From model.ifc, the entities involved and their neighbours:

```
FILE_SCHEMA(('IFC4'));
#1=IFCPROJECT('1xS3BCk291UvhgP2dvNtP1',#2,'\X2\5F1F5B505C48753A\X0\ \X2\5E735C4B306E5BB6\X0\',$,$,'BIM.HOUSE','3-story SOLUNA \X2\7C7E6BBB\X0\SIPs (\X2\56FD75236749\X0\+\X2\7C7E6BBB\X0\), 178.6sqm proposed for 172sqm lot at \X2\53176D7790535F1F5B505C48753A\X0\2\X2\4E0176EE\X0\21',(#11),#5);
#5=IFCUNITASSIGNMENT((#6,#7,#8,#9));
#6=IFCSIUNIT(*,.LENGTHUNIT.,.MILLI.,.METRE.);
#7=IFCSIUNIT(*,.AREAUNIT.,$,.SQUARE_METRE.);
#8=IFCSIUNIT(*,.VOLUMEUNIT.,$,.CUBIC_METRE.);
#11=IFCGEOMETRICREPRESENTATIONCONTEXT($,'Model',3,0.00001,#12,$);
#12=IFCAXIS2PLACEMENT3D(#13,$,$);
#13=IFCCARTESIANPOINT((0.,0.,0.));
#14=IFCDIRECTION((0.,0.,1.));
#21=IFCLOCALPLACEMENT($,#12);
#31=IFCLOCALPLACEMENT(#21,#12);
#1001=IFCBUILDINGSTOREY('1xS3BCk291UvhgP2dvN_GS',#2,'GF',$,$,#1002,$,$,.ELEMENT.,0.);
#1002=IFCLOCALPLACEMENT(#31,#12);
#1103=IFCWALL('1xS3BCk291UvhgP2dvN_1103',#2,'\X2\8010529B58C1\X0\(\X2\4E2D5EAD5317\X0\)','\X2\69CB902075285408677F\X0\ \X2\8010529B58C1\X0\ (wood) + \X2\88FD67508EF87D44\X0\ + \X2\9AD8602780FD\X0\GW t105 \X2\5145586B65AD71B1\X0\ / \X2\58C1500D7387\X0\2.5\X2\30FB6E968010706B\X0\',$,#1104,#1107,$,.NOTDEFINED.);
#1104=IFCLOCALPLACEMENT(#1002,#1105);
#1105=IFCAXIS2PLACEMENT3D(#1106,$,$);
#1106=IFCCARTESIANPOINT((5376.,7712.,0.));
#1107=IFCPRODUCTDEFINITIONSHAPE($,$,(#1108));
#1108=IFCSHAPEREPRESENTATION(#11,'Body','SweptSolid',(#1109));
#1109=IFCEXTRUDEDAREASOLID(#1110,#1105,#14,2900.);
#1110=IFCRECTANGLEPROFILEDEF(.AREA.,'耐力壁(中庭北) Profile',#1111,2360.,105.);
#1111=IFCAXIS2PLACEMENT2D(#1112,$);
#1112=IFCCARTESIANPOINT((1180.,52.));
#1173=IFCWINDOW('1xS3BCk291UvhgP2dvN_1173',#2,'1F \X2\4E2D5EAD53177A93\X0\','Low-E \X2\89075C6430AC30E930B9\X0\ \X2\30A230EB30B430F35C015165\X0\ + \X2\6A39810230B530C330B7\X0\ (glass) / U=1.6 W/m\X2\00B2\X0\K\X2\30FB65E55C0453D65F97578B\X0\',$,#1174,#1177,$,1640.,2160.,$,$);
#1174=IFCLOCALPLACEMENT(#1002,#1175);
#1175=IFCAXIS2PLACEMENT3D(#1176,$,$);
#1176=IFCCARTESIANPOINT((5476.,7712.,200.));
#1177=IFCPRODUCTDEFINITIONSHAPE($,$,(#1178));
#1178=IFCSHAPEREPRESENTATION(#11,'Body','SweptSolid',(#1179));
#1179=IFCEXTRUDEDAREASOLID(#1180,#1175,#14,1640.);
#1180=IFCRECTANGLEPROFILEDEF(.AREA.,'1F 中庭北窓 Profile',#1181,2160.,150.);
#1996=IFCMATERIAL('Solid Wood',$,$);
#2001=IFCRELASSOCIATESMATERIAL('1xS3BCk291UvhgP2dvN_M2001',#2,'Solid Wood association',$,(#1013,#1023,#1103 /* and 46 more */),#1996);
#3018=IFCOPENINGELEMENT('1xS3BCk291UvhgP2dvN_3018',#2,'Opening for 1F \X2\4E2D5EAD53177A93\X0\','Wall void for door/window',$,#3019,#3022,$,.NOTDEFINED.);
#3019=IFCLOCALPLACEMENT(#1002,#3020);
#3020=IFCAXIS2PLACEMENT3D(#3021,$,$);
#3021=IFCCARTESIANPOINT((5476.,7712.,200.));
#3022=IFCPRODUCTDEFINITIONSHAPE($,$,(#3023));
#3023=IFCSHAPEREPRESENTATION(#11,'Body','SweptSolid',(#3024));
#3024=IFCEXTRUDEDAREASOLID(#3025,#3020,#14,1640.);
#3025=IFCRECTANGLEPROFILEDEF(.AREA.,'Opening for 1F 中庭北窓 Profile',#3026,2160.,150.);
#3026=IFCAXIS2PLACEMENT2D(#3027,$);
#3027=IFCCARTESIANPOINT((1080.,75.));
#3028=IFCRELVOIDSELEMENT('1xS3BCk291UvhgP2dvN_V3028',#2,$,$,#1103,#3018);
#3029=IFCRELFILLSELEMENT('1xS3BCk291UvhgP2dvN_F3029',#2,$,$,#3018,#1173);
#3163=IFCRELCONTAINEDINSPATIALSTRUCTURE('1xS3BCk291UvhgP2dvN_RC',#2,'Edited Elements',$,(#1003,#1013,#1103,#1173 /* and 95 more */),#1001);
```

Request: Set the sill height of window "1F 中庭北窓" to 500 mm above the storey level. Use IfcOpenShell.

```python
import numpy as np
import ifcopenshell
import ifcopenshell.api.geometry
import ifcopenshell.geom
import ifcopenshell.util.element
import ifcopenshell.util.placement
import ifcopenshell.util.shape
import ifcopenshell.util.unit

model = ifcopenshell.open("model.ifc")
unit_scale = ifcopenshell.util.unit.calculate_unit_scale(model)

window = model.by_guid("1xS3BCk291UvhgP2dvN_1173")
opening = window.FillsVoids[0].RelatingOpeningElement
storey = ifcopenshell.util.element.get_container(window, ifc_class="IfcBuildingStorey")
level = ifcopenshell.util.placement.get_local_placement(storey.ObjectPlacement)[2, 3]

# The opening's origin need not be at the sill, so measure its lowest point.
shape = ifcopenshell.geom.create_shape(ifcopenshell.geom.settings(), opening)
bottom = ifcopenshell.util.shape.get_shape_bottom_elevation(shape, shape.geometry) / unit_scale
dz = level + 0.5 / unit_scale - bottom

shift = np.array([0.0, 0.0, dz])
# The window is not placed relative to its opening, so move both.
for product in (opening, window):
    matrix = ifcopenshell.util.placement.get_local_placement(product.ObjectPlacement)
    matrix[:3, 3] += shift
    ifcopenshell.api.geometry.edit_object_placement(model, product=product, matrix=matrix, is_si=False)

print(f"moved by {dz * unit_scale:+.3f} m")

model.write("model-out.ifc")
```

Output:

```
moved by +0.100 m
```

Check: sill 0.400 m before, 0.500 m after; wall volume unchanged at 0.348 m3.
